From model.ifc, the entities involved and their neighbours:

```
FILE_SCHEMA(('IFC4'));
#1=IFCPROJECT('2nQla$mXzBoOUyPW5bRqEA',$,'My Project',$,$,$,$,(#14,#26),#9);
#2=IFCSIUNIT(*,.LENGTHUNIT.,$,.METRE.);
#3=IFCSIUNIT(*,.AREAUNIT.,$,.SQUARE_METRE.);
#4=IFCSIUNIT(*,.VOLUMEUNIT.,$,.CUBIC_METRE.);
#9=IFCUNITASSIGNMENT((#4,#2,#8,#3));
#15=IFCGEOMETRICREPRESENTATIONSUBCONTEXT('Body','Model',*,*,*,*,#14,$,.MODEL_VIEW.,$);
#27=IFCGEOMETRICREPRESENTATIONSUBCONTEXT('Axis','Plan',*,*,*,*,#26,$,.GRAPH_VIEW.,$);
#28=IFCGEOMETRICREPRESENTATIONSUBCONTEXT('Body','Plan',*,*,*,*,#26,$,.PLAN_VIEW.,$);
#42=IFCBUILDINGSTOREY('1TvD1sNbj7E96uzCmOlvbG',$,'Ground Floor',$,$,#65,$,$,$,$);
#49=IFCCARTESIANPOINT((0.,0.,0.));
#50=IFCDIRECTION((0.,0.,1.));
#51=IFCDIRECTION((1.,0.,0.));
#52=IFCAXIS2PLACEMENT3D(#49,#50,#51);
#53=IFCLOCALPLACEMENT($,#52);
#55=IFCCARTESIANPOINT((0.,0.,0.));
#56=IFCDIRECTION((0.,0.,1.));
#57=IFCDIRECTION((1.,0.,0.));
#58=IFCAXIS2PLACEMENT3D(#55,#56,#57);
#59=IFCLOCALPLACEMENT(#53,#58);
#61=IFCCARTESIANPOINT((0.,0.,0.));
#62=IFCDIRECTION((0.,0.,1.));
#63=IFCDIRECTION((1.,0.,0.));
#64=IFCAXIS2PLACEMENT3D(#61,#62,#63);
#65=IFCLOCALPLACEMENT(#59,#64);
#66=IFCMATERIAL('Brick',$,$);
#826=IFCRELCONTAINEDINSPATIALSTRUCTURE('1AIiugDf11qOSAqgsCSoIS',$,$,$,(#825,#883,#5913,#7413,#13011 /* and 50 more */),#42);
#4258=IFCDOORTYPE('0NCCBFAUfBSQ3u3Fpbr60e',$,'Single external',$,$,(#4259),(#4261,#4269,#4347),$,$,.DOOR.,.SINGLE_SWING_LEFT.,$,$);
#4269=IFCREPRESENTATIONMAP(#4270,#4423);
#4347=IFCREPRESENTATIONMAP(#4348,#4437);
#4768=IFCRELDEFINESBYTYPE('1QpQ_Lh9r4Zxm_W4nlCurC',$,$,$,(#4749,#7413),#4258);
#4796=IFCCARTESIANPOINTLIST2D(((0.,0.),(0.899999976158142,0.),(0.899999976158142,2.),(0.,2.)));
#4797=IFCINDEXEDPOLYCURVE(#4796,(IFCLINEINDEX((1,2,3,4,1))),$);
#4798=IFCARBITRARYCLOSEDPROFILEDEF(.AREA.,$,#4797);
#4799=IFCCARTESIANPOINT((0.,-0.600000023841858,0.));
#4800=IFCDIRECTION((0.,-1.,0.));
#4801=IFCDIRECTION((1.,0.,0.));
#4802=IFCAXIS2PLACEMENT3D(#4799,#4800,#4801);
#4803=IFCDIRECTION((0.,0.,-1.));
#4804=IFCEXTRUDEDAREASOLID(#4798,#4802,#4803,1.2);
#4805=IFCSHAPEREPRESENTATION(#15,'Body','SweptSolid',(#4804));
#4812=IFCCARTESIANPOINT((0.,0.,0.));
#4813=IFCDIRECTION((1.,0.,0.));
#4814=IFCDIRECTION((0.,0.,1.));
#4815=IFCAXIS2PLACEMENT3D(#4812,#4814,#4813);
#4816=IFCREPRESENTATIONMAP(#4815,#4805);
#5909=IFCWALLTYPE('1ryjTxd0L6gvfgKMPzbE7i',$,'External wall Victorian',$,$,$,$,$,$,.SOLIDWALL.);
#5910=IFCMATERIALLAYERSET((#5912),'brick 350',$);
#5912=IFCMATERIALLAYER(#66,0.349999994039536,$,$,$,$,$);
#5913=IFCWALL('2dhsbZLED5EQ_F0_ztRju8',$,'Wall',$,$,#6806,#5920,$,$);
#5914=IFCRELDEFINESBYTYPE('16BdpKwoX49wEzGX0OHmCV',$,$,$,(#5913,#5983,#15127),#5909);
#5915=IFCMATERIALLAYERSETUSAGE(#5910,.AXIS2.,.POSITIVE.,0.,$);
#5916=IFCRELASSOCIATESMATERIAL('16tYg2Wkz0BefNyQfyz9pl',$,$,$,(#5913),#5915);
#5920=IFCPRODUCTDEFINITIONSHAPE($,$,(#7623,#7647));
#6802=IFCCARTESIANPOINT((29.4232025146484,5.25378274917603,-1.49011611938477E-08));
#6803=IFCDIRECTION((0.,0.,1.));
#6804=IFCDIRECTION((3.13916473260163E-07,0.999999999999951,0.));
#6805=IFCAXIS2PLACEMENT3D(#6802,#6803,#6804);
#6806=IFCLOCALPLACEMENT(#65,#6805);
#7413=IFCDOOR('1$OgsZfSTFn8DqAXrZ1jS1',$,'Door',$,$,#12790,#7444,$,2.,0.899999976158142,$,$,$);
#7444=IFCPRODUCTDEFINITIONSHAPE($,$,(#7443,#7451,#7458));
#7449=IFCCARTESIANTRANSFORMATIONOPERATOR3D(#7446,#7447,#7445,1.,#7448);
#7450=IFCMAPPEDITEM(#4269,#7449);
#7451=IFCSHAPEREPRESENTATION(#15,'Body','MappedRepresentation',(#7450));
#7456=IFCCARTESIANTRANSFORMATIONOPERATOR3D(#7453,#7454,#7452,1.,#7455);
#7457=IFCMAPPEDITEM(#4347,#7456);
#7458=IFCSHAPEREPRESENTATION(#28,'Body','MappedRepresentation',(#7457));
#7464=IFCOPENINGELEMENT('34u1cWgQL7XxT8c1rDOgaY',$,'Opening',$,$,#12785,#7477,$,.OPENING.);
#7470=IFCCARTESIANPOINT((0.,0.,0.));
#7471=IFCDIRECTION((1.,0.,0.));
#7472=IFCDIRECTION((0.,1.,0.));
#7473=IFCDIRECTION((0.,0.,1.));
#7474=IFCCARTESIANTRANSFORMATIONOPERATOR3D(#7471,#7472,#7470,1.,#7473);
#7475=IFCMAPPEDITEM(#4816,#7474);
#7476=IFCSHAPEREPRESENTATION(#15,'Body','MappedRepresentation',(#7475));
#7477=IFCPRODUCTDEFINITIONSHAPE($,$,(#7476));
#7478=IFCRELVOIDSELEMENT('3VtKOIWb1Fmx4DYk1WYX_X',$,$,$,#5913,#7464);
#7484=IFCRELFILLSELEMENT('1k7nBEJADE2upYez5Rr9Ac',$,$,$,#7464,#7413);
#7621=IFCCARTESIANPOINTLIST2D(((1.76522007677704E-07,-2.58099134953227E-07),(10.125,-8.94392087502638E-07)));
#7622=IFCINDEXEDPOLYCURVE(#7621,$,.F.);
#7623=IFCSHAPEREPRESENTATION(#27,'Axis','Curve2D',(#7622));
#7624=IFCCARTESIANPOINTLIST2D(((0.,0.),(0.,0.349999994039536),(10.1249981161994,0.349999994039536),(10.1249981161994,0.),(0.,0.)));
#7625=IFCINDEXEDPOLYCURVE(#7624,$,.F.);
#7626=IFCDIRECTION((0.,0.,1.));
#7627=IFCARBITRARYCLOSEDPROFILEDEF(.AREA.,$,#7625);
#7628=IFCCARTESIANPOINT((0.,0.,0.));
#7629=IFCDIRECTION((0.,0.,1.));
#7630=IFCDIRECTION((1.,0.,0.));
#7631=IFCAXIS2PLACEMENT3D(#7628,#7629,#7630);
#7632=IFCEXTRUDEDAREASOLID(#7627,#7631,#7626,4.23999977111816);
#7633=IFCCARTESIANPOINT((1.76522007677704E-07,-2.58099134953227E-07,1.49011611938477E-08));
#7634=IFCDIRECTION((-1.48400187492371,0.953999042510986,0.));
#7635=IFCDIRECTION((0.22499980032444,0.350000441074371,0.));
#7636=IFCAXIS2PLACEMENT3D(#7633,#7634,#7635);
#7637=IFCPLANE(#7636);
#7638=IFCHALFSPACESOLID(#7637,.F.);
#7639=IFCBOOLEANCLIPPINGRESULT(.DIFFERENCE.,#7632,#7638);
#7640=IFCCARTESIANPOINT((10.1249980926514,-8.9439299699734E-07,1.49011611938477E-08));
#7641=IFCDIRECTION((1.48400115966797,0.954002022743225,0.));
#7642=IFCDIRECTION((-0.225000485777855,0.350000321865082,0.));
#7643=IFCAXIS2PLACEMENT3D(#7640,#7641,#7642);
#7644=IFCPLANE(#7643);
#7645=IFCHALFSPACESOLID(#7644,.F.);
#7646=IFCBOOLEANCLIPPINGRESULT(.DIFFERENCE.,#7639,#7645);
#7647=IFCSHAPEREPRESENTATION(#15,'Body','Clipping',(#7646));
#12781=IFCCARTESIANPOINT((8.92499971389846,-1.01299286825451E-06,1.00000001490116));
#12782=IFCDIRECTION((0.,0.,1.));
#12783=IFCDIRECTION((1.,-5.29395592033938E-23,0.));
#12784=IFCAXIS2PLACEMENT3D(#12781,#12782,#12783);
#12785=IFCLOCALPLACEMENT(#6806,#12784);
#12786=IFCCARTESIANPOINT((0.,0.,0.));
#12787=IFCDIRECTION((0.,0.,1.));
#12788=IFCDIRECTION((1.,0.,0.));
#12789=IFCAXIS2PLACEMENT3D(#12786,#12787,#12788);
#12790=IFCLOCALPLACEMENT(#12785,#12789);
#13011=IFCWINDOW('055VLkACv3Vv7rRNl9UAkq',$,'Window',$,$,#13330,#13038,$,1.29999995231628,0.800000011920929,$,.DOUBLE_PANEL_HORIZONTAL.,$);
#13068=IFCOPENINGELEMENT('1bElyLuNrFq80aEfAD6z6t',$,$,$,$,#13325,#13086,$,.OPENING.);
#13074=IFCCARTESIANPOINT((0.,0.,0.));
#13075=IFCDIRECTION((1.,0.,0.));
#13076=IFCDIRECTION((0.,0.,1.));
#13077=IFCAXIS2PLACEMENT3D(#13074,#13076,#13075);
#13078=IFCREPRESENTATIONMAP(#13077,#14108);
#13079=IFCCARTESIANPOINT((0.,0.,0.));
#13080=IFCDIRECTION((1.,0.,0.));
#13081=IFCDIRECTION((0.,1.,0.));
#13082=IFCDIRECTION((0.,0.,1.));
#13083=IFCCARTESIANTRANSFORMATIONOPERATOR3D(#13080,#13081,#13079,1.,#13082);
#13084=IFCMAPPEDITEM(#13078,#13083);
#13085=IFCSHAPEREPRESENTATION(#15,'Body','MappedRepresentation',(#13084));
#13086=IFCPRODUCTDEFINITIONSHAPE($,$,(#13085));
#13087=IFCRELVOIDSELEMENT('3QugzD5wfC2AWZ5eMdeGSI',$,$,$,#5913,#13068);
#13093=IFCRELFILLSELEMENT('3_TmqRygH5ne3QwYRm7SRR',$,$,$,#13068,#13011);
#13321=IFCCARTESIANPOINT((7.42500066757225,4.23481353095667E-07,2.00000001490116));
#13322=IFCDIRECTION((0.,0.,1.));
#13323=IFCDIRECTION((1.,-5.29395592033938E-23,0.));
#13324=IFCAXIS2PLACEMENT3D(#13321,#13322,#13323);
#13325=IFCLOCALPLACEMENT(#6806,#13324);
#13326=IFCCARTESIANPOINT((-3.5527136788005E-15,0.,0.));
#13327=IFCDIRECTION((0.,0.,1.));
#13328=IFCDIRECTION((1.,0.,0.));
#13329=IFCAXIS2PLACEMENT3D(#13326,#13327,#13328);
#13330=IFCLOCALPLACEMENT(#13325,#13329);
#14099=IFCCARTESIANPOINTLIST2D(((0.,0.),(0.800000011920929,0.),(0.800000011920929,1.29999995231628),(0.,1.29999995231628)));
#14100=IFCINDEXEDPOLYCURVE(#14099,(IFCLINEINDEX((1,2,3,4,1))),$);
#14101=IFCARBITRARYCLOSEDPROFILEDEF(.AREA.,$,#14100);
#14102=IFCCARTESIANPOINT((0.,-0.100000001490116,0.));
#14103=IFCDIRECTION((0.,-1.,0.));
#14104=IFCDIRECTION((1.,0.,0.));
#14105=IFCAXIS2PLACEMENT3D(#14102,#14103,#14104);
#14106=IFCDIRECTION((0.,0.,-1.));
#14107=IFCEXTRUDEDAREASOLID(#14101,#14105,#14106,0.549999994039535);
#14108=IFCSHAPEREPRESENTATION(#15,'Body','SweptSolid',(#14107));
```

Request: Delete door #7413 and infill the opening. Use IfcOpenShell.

```python
import ifcopenshell
import ifcopenshell.api.feature
import ifcopenshell.api.root
import ifcopenshell.geom
import ifcopenshell.util.shape

model = ifcopenshell.open("model.ifc")
settings = ifcopenshell.geom.settings()


def volume(element):
    """Net volume in cubic metres, openings subtracted."""
    shape = ifcopenshell.geom.create_shape(settings, element)
    return ifcopenshell.util.shape.get_volume(shape.geometry)


door = model.by_guid("1$OgsZfSTFn8DqAXrZ1jS1")
opening = door.FillsVoids[0].RelatingOpeningElement
wall = opening.VoidsElements[0].RelatingBuildingElement
before = volume(wall)

ifcopenshell.api.root.remove_product(model, product=door)
ifcopenshell.api.feature.remove_feature(model, feature=opening)

after = volume(wall)

print(f"wall volume {before:.3f} -> {after:.3f} m3")

model.write("model_updated.ifc")
```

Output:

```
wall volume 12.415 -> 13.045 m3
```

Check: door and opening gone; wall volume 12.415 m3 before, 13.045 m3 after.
